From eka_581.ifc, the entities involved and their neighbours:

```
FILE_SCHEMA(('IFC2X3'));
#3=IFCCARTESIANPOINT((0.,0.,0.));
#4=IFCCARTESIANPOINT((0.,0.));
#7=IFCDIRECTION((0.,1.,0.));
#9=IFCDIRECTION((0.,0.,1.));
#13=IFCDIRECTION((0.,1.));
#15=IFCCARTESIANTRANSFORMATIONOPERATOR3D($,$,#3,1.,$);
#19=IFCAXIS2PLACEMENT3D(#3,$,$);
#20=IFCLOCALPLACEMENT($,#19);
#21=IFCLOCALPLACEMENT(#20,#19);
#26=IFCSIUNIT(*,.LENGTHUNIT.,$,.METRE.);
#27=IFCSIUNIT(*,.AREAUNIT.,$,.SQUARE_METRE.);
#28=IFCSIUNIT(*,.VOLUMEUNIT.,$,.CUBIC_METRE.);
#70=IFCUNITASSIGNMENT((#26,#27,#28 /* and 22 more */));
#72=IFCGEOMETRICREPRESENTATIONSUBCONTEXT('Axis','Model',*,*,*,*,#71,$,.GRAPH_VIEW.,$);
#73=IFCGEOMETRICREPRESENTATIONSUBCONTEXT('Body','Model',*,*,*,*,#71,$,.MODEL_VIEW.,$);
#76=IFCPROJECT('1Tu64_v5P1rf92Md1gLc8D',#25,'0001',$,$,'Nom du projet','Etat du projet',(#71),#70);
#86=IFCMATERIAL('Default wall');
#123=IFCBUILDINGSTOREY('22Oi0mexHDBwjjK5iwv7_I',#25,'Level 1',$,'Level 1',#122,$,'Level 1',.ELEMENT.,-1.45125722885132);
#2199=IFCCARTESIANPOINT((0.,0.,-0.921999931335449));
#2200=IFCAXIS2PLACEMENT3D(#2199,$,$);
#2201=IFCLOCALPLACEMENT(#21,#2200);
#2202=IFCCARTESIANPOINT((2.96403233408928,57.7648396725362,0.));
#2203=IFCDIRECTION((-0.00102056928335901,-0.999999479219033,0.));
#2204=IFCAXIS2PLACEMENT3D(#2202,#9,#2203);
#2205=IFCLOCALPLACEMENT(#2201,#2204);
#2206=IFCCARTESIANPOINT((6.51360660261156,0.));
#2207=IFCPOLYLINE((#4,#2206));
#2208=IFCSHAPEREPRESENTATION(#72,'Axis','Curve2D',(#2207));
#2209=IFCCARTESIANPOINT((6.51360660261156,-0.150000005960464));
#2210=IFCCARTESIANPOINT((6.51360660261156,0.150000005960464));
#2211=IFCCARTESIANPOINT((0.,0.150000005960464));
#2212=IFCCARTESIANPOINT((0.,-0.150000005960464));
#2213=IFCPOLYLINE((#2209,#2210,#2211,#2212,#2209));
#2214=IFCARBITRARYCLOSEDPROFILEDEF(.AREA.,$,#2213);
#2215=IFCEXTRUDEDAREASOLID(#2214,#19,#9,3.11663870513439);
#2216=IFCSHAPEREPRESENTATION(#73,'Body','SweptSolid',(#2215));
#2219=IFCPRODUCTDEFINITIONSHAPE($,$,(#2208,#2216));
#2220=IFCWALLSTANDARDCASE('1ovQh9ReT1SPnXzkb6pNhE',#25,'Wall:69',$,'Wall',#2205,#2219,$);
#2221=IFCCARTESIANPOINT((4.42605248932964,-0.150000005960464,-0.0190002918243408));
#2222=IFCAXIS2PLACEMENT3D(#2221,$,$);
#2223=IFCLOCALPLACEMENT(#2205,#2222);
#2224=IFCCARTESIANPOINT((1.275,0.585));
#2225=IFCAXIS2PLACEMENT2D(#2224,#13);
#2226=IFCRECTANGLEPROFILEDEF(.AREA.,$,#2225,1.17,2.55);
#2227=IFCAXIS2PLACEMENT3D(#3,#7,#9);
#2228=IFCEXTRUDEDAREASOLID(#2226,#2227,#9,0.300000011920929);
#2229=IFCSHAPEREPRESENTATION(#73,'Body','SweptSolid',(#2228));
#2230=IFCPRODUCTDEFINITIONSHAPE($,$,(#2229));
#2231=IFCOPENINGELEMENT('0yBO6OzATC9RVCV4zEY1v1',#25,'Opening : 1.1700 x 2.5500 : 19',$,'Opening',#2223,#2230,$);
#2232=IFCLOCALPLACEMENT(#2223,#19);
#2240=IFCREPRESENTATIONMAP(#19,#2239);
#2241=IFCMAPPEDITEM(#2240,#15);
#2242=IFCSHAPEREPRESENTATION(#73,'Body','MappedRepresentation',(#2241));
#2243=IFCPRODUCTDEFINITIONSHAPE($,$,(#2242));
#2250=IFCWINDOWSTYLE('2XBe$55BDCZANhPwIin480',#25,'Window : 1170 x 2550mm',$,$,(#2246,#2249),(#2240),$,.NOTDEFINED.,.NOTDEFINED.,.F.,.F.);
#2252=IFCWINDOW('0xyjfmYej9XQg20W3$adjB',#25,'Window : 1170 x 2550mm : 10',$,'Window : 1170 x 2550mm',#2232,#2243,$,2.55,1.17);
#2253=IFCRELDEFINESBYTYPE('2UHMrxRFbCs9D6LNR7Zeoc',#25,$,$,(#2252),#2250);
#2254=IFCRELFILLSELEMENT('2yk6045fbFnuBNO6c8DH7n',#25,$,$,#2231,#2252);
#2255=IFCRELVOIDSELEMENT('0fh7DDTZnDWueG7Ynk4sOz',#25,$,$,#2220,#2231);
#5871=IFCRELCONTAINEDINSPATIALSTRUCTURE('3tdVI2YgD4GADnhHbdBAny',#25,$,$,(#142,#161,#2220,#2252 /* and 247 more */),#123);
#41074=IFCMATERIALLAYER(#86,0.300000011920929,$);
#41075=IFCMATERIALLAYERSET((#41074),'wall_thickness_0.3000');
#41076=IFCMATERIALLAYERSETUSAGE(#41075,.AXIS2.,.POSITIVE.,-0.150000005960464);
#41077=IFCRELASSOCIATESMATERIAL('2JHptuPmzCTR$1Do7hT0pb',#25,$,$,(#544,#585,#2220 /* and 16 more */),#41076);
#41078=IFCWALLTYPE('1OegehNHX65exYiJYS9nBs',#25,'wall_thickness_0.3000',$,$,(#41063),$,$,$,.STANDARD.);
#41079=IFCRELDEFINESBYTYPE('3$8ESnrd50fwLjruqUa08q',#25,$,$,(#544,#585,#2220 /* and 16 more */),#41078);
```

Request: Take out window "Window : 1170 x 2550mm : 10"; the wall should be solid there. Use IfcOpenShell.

```python
import ifcopenshell
import ifcopenshell.api.feature
import ifcopenshell.api.root
import ifcopenshell.geom
import ifcopenshell.util.shape

model = ifcopenshell.open("eka_581.ifc")
settings = ifcopenshell.geom.settings()


def volume(element):
    """Net volume in cubic metres, openings subtracted."""
    shape = ifcopenshell.geom.create_shape(settings, element)
    return ifcopenshell.util.shape.get_volume(shape.geometry)


window = model.by_guid("0xyjfmYej9XQg20W3$adjB")
opening = window.FillsVoids[0].RelatingOpeningElement
wall = opening.VoidsElements[0].RelatingBuildingElement
before = volume(wall)

ifcopenshell.api.root.remove_product(model, product=window)
ifcopenshell.api.feature.remove_feature(model, feature=opening)

after = volume(wall)

print(f"wall volume {before:.3f} -> {after:.3f} m3")

model.write("eka_581-out.ifc")
```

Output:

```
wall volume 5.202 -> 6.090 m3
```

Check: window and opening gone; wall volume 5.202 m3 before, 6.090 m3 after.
